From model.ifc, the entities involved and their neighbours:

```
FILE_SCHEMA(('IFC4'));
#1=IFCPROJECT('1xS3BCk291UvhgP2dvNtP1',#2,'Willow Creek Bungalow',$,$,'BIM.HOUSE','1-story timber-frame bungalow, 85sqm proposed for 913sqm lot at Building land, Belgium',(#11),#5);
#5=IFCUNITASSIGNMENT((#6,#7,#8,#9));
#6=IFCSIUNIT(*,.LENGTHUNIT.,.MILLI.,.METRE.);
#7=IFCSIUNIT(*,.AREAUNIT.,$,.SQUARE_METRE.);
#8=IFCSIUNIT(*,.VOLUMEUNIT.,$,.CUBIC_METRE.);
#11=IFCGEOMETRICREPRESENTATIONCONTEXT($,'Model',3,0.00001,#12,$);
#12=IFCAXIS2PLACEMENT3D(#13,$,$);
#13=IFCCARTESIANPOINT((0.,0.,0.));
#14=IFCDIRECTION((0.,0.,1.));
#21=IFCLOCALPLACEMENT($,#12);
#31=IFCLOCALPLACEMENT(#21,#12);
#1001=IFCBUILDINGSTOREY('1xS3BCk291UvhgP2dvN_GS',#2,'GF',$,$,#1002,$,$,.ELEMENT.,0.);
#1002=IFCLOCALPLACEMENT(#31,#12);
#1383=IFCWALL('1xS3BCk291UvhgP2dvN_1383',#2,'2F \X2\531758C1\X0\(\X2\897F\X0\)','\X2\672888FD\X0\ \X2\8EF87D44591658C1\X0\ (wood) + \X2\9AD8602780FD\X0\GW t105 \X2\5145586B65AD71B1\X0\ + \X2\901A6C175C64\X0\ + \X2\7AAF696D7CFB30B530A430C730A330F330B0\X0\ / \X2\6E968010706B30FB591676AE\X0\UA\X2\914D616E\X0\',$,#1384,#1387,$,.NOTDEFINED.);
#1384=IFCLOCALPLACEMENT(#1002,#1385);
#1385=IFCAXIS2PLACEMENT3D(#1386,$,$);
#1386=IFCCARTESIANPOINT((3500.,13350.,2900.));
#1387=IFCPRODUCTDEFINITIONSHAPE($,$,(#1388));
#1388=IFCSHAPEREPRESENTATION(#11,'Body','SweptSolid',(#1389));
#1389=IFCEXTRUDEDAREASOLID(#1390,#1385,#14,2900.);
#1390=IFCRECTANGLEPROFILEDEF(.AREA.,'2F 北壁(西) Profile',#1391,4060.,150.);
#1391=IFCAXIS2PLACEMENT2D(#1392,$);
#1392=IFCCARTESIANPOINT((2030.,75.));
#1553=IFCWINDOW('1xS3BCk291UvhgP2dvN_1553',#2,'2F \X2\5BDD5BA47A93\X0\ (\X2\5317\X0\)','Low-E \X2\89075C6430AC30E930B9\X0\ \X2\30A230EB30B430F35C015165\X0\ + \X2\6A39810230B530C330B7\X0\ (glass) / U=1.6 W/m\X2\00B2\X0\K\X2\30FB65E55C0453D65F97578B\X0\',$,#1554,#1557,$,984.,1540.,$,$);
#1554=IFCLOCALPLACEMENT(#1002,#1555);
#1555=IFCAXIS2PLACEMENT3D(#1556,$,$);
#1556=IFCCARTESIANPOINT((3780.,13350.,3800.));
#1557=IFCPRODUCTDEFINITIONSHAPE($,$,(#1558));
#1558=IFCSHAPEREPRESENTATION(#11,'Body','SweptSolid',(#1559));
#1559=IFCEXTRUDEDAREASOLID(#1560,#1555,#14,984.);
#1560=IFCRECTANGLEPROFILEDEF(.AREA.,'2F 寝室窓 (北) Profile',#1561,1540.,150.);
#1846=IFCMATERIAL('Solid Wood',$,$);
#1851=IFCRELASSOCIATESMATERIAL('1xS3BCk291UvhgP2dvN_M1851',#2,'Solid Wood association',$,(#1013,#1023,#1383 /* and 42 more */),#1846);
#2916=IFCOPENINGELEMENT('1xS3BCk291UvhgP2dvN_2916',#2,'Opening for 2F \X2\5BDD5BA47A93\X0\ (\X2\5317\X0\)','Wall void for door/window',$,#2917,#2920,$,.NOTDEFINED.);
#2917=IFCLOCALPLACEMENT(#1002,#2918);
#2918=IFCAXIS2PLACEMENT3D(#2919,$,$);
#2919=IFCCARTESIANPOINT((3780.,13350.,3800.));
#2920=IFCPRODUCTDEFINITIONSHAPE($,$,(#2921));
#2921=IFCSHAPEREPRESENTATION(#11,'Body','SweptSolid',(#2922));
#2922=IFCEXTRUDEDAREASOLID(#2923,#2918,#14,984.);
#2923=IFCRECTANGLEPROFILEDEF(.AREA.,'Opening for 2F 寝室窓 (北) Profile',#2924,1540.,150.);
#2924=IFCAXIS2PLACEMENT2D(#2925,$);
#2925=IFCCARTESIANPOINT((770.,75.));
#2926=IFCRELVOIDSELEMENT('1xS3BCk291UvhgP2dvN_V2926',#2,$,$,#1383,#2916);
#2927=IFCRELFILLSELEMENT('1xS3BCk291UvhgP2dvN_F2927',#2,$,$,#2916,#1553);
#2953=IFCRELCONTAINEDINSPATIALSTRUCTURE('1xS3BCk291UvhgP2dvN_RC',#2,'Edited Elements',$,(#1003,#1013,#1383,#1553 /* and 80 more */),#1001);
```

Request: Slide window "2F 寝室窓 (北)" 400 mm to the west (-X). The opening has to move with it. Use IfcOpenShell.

```python
import ifcopenshell
import ifcopenshell.api.geometry
import ifcopenshell.util.placement
import ifcopenshell.util.unit

model = ifcopenshell.open("model.ifc")
unit_scale = ifcopenshell.util.unit.calculate_unit_scale(model)

window = model.by_guid("1xS3BCk291UvhgP2dvN_1553")
opening = window.FillsVoids[0].RelatingOpeningElement
wall = opening.VoidsElements[0].RelatingBuildingElement

wall_matrix = ifcopenshell.util.placement.get_local_placement(wall.ObjectPlacement)
shift = wall_matrix[:3, 0] * -0.4 / unit_scale
before = ifcopenshell.util.placement.get_local_placement(window.ObjectPlacement)[:3, 3].copy()

# The window is not placed relative to its opening, so move both.
for product in (opening, window):
    matrix = ifcopenshell.util.placement.get_local_placement(product.ObjectPlacement)
    matrix[:3, 3] += shift
    ifcopenshell.api.geometry.edit_object_placement(model, product=product, matrix=matrix, is_si=False)

after = ifcopenshell.util.placement.get_local_placement(window.ObjectPlacement)[:3, 3]
print("window moved by", (after - before).round(3) + 0.0)

model.write("model_edited.ifc")
```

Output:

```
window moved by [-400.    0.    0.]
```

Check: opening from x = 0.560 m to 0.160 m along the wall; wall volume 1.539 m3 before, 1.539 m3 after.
